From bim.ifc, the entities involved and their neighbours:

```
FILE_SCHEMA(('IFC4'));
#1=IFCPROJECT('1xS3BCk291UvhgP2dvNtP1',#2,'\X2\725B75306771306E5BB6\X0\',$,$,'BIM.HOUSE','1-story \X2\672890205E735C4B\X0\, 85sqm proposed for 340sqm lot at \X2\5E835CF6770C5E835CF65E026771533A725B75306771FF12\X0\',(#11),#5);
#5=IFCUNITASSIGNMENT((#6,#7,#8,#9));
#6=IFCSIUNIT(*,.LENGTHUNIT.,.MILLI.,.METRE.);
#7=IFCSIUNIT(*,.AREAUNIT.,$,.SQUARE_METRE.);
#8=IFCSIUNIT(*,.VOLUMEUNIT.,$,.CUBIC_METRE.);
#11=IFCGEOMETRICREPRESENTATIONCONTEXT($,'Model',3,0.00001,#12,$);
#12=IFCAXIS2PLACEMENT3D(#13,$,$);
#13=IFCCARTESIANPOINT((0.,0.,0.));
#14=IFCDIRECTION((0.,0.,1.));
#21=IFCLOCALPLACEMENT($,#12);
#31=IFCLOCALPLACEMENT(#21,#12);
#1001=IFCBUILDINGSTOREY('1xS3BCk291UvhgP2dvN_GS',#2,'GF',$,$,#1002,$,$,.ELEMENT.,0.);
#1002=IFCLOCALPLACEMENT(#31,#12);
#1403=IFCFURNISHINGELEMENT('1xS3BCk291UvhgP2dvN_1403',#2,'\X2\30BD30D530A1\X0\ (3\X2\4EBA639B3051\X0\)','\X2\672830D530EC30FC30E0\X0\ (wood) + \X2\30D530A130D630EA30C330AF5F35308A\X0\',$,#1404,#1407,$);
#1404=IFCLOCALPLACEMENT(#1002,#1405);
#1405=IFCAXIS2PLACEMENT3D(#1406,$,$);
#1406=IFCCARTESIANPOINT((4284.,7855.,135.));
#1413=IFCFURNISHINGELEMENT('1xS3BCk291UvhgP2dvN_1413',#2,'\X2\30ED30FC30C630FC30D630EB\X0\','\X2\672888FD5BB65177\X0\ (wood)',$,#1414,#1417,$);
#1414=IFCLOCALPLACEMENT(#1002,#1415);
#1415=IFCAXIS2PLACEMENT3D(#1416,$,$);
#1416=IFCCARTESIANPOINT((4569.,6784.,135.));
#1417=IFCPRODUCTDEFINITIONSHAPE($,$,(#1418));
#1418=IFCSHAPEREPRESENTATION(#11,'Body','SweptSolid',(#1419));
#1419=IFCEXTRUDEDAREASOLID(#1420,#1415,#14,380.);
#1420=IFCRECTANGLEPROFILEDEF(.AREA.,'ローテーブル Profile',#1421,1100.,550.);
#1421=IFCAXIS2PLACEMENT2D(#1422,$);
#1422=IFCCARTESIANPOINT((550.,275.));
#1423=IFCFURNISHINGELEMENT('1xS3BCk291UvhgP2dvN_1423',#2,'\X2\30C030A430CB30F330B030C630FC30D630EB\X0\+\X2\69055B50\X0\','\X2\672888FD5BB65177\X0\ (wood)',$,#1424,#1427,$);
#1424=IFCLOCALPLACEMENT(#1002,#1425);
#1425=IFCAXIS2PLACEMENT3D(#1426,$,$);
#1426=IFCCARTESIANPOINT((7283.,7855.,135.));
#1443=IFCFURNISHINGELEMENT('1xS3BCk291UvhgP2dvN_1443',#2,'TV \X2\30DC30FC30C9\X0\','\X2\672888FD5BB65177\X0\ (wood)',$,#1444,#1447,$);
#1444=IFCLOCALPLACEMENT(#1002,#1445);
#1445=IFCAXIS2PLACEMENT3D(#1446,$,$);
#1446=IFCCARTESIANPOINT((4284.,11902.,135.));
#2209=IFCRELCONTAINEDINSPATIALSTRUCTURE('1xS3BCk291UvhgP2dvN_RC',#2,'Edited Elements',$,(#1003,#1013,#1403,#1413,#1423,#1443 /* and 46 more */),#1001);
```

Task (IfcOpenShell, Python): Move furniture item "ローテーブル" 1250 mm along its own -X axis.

```python
import ifcopenshell
import ifcopenshell.api.geometry
import ifcopenshell.util.placement
import ifcopenshell.util.unit

model = ifcopenshell.open("bim.ifc")
unit_scale = ifcopenshell.util.unit.calculate_unit_scale(model)

item = model.by_guid("1xS3BCk291UvhgP2dvN_1413")
matrix = ifcopenshell.util.placement.get_local_placement(item.ObjectPlacement)
matrix[:3, 3] -= matrix[:3, 0] * 1.25 / unit_scale
ifcopenshell.api.geometry.edit_object_placement(model, product=item, matrix=matrix, is_si=False)

print(ifcopenshell.util.placement.get_local_placement(item.ObjectPlacement).round(3) + 0.0)

model.write("bim_edited.ifc")
```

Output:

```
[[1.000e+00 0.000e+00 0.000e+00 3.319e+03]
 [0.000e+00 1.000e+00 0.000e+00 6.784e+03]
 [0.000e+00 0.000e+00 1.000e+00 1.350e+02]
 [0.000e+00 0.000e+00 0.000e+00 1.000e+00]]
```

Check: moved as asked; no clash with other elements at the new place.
